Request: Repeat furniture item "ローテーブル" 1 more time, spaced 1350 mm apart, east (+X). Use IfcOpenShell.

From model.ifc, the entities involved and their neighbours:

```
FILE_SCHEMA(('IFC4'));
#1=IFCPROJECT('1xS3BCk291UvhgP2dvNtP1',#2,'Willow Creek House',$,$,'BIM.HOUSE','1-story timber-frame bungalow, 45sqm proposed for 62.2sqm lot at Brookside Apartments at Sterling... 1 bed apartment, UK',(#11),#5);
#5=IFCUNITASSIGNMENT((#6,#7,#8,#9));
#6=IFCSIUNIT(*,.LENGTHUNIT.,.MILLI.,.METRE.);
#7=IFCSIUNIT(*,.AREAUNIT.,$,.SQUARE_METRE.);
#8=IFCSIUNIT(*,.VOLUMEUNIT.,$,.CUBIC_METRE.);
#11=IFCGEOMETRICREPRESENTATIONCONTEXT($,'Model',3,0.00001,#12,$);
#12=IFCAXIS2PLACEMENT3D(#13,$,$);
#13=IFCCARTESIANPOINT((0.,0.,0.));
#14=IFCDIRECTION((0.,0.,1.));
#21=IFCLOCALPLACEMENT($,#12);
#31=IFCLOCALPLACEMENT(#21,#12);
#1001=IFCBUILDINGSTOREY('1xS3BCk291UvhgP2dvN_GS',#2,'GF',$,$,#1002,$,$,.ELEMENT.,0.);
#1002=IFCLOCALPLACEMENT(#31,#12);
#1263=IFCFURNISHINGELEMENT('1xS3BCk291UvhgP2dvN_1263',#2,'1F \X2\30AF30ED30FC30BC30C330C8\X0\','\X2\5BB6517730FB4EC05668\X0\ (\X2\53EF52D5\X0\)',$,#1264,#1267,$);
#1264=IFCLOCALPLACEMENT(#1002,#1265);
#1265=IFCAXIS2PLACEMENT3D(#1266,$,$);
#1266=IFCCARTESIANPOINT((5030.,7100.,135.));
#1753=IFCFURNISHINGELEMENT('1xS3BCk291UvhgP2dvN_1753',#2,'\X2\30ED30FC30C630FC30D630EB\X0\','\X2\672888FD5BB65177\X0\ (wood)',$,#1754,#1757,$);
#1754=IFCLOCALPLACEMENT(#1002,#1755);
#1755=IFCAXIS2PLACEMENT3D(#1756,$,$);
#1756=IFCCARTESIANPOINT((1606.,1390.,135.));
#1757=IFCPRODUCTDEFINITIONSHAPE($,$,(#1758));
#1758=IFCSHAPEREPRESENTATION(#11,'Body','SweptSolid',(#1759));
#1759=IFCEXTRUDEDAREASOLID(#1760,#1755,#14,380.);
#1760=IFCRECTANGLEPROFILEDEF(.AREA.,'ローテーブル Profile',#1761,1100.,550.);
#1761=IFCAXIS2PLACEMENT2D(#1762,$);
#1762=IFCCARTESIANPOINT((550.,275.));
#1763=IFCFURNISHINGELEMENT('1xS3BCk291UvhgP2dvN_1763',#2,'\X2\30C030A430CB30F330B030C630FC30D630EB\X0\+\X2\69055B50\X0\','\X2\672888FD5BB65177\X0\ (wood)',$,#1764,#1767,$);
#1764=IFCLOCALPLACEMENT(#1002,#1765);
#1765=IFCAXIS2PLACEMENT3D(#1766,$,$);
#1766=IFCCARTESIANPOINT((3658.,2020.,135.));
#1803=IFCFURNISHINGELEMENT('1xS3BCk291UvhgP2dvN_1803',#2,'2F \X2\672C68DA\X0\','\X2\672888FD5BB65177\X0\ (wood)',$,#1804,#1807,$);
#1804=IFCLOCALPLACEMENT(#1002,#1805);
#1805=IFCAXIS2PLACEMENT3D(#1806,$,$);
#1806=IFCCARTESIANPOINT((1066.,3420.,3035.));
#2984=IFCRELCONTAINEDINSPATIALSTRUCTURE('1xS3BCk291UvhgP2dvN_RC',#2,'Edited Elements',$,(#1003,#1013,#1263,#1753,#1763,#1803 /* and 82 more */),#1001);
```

```python
import numpy as np
import ifcopenshell
import ifcopenshell.api.geometry
import ifcopenshell.api.root
import ifcopenshell.util.element
import ifcopenshell.util.placement
import ifcopenshell.util.unit

model = ifcopenshell.open("model.ifc")
unit_scale = ifcopenshell.util.unit.calculate_unit_scale(model)


def reuse_history(source, copy):
    """copy_class also copies each property set's owner history, people and application; keep the originals."""
    for rel in copy.IsDefinedBy:
        if rel.is_a("IfcRelDefinesByProperties") and (history := rel.RelatingPropertyDefinition.OwnerHistory):
            rel.RelatingPropertyDefinition.OwnerHistory = source.OwnerHistory
            ifcopenshell.util.element.remove_deep2(model, history)


source = model.by_guid("1xS3BCk291UvhgP2dvN_1753")
base = ifcopenshell.util.placement.get_local_placement(source.ObjectPlacement)
step = np.array([1.0, 0.0, 0.0]) * 1.35 / unit_scale

for i in range(1, 2):
    copy = ifcopenshell.api.root.copy_class(model, product=source)
    copy.Representation = ifcopenshell.util.element.copy_deep(
        model, source.Representation, exclude=["IfcGeometricRepresentationContext", "IfcRepresentationMap"]
    )
    reuse_history(source, copy)
    matrix = base.copy()
    matrix[:3, 3] += i * step
    print("added at", matrix[:3, 3].round(3) + 0.0)
    ifcopenshell.api.geometry.edit_object_placement(model, product=copy, matrix=matrix, is_si=False)

model.write("model_rev.ifc")
```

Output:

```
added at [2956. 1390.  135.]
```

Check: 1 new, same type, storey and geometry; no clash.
